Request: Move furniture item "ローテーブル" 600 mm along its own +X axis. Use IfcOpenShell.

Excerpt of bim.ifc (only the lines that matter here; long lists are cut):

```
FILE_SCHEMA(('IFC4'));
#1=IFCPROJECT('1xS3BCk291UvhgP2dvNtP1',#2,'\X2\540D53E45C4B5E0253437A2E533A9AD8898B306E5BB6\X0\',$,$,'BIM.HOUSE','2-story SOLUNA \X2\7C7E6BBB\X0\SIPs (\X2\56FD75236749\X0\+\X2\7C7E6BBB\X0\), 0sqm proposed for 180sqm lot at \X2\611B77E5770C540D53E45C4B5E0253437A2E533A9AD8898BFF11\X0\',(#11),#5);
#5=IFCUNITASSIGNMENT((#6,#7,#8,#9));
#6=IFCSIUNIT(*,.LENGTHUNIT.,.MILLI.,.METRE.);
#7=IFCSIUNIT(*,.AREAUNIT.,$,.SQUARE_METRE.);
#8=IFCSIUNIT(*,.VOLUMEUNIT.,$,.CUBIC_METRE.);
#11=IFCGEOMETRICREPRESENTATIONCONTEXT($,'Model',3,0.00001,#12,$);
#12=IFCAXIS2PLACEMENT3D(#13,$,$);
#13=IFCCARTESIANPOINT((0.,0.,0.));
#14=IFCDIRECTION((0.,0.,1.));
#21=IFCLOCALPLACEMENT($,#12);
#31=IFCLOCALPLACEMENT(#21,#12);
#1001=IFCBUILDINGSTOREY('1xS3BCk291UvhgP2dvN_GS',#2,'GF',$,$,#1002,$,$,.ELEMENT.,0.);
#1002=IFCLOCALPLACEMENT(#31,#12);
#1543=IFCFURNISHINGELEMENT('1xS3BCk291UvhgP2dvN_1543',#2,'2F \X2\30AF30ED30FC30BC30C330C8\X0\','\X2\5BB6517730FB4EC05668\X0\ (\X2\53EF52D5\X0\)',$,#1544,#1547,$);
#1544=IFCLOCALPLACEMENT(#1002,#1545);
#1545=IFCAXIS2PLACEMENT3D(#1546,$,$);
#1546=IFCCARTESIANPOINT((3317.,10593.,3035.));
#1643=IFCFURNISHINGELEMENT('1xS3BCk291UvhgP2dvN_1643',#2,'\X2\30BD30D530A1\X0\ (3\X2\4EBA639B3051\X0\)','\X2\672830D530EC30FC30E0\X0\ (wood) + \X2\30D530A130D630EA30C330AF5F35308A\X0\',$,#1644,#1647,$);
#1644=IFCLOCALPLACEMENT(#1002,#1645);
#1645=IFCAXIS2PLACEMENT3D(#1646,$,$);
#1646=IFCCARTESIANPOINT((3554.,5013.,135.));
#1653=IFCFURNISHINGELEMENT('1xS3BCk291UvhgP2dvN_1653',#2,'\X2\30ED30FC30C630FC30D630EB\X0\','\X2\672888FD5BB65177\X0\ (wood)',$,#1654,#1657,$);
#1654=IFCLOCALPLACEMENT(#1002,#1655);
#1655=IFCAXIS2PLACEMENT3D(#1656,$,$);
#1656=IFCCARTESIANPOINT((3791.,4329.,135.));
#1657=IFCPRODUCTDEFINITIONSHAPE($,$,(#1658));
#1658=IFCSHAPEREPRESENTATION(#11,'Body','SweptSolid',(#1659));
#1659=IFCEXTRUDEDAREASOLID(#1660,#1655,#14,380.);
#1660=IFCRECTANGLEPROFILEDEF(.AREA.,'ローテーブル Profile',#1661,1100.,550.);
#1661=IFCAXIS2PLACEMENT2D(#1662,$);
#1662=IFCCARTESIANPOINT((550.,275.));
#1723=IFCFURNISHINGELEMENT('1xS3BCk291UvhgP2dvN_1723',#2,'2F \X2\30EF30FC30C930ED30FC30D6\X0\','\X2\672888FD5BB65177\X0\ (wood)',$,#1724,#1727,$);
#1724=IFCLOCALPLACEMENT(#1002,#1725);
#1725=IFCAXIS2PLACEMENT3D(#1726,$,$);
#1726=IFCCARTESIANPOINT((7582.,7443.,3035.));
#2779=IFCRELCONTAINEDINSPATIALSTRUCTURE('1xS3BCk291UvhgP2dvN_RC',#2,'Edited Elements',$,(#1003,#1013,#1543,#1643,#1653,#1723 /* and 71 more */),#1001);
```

```python
import ifcopenshell
import ifcopenshell.api.geometry
import ifcopenshell.util.placement
import ifcopenshell.util.unit

model = ifcopenshell.open("bim.ifc")
unit_scale = ifcopenshell.util.unit.calculate_unit_scale(model)

item = model.by_guid("1xS3BCk291UvhgP2dvN_1653")
matrix = ifcopenshell.util.placement.get_local_placement(item.ObjectPlacement)
matrix[:3, 3] += matrix[:3, 0] * 0.6 / unit_scale
ifcopenshell.api.geometry.edit_object_placement(model, product=item, matrix=matrix, is_si=False)

print(ifcopenshell.util.placement.get_local_placement(item.ObjectPlacement).round(3) + 0.0)

model.write("bim-out.ifc")
```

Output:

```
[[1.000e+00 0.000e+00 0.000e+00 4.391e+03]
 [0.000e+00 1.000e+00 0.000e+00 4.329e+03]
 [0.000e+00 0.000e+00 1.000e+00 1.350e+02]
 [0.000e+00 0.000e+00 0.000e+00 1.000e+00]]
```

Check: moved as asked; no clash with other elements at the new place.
